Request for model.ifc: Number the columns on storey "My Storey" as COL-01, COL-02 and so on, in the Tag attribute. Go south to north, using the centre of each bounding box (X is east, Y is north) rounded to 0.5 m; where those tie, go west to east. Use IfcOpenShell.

First a look at what the model holds.

```python
import ifcopenshell
import ifcopenshell.util.element
import ifcopenshell.util.placement

model = ifcopenshell.open("model.ifc")
print(model.schema)
storey = next(s for s in model.by_type("IfcBuildingStorey") if s.Name == "My Storey")
columns = [e for e in ifcopenshell.util.element.get_decomposition(storey) if e.is_a("IfcColumn")]
for e in sorted(columns, key=lambda e: e.id()):
    origin = ifcopenshell.util.placement.get_local_placement(e.ObjectPlacement)[:3, 3]
    print(e.id(), e.Tag, e.Name, origin.round(2) + 0.0, sep=" | ")
```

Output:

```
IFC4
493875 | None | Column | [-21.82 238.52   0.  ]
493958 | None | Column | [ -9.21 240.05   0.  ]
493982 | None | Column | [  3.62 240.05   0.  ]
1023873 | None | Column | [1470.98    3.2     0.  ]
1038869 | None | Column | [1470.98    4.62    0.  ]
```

```python
import ifcopenshell
import ifcopenshell.geom
import ifcopenshell.util.element
import ifcopenshell.util.shape

model = ifcopenshell.open("model.ifc")
settings = ifcopenshell.geom.settings()
settings.set("use-world-coords", True)


def centre(element):
    shape = ifcopenshell.geom.create_shape(settings, element)
    return ifcopenshell.util.shape.get_bbox_centroid(shape.geometry)


storey = next(s for s in model.by_type("IfcBuildingStorey") if s.Name == "My Storey")
columns = [e for e in ifcopenshell.util.element.get_decomposition(storey) if e.is_a("IfcColumn")]

# Insertion points can sit at a corner or the storey origin, so sort by the geometry (in metres).
centres = {e: centre(e) for e in columns}
columns.sort(key=lambda e: (round(centres[e][1] / 0.5), centres[e][0]))

for i, e in enumerate(columns, start=1):
    number = f"COL-{i:02d}"
    e.Tag = number
    print(e.id(), number)

model.write("model_v2.ifc")
```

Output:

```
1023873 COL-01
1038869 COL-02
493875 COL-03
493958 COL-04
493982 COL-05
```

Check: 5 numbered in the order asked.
